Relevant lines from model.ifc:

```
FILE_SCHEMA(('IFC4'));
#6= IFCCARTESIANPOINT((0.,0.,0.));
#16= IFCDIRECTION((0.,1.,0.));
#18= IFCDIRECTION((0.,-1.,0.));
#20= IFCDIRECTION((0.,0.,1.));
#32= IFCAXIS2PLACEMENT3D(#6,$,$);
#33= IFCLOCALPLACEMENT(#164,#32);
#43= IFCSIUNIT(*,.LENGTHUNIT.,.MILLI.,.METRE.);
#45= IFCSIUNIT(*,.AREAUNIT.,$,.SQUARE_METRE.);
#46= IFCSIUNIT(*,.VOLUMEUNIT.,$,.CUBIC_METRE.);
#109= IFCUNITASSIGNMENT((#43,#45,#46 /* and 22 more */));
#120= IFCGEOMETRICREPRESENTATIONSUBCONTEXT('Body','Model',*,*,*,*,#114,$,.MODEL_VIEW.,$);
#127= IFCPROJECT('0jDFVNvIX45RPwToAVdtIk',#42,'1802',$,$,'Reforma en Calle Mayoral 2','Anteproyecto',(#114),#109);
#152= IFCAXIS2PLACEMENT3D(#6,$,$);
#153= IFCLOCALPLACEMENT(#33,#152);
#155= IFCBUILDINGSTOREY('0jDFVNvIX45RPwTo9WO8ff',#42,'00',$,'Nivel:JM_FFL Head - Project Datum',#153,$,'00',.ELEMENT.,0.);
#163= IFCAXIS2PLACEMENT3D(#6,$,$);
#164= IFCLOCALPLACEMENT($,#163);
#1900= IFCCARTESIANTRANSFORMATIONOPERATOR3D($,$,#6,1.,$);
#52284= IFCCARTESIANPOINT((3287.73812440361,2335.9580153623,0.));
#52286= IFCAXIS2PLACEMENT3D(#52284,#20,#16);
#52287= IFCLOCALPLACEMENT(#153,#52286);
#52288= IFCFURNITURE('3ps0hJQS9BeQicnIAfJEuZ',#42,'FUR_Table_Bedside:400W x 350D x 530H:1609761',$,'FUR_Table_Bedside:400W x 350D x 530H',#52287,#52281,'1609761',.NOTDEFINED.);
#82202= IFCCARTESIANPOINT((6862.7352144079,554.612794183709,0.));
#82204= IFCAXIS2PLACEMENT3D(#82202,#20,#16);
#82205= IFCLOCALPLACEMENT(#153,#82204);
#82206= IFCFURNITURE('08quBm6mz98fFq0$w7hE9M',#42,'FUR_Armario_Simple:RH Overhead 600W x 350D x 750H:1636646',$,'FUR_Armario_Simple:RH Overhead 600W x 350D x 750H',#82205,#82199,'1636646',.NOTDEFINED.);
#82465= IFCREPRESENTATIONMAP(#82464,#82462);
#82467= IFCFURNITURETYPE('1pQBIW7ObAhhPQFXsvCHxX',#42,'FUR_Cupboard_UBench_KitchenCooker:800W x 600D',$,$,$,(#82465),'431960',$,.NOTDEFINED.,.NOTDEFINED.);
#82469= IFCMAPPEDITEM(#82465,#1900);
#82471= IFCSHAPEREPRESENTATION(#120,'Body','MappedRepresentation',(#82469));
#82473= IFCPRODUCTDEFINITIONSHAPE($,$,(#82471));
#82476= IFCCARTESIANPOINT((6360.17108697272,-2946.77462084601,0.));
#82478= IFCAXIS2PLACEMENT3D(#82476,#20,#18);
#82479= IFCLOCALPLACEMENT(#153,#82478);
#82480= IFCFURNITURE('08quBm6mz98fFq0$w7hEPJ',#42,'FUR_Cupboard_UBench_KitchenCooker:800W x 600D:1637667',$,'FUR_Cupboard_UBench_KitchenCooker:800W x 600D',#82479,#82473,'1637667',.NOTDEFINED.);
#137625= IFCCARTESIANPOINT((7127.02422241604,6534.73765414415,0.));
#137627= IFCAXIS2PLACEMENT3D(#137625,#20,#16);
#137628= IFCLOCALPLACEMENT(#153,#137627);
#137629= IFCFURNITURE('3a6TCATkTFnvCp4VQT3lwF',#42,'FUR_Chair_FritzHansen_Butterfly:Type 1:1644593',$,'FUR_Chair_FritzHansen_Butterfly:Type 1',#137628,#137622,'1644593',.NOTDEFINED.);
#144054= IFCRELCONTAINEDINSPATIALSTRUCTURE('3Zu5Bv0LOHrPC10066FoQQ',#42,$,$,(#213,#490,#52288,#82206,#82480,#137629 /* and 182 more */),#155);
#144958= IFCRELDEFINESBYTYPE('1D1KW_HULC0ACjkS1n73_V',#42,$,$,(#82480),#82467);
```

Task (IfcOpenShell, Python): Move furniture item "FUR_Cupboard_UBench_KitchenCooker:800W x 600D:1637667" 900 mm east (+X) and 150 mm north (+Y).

```python
import ifcopenshell
import ifcopenshell.api.geometry
import ifcopenshell.util.placement
import ifcopenshell.util.unit

model = ifcopenshell.open("model.ifc")
unit_scale = ifcopenshell.util.unit.calculate_unit_scale(model)

item = model.by_guid("08quBm6mz98fFq0$w7hEPJ")
matrix = ifcopenshell.util.placement.get_local_placement(item.ObjectPlacement)
matrix[0, 3] += 0.9 / unit_scale
matrix[1, 3] += 0.15 / unit_scale
ifcopenshell.api.geometry.edit_object_placement(model, product=item, matrix=matrix, is_si=False)

print(ifcopenshell.util.placement.get_local_placement(item.ObjectPlacement).round(3) + 0.0)

model.write("model_edited.ifc")
```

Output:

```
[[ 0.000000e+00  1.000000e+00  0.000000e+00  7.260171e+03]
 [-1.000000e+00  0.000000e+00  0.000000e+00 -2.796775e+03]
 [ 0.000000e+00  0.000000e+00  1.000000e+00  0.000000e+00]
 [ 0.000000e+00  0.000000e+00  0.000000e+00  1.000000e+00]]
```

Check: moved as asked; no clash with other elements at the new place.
